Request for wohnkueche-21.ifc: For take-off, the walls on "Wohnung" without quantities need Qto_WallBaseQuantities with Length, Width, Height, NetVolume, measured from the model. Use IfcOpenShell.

First a look at what the model holds.

```python
import ifcopenshell
import ifcopenshell.util.element
import ifcopenshell.util.unit

model = ifcopenshell.open("wohnkueche-21.ifc")
print(model.schema)
for unit_type in ("LENGTHUNIT", "AREAUNIT", "VOLUMEUNIT"):
    print(unit_type, ifcopenshell.util.unit.calculate_unit_scale(model, unit_type))
storey = next(s for s in model.by_type("IfcBuildingStorey") if s.Name == "Wohnung")
walls = [e for e in ifcopenshell.util.element.get_decomposition(storey) if e.is_a("IfcWall")]
for e in sorted(walls, key=lambda e: e.id()):
    print(e.id(), e.is_a(), e.Name, list(ifcopenshell.util.element.get_psets(e, qtos_only=True)), sep=" | ")
```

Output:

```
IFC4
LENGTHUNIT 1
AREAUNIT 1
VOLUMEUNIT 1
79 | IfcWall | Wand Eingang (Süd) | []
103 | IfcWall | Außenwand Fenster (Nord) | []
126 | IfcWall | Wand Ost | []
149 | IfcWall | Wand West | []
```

```python
import ifcopenshell
import ifcopenshell.api.pset
import ifcopenshell.geom
import ifcopenshell.util.element
import ifcopenshell.util.shape
import ifcopenshell.util.unit

model = ifcopenshell.open("wohnkueche-21.ifc")
unit_scale = ifcopenshell.util.unit.calculate_unit_scale(model)
volume_scale = ifcopenshell.util.unit.calculate_unit_scale(model, "VOLUMEUNIT")
settings = ifcopenshell.geom.settings()

storey = next(s for s in model.by_type("IfcBuildingStorey") if s.Name == "Wohnung")
walls = [e for e in ifcopenshell.util.element.get_decomposition(storey) if e.is_a("IfcWall")]

for e in sorted(walls, key=lambda e: e.id()):
    if ifcopenshell.util.element.get_psets(e, qtos_only=True, should_inherit=False):
        continue
    # Geometry comes back in metres, in the element's own axes.
    shape = ifcopenshell.geom.create_shape(settings, e)
    values = {
        "Length": ifcopenshell.util.shape.get_x(shape.geometry) / unit_scale,
        "Width": ifcopenshell.util.shape.get_y(shape.geometry) / unit_scale,
        "Height": ifcopenshell.util.shape.get_z(shape.geometry) / unit_scale,
        "NetVolume": ifcopenshell.util.shape.get_volume(shape.geometry) / volume_scale,
    }
    qto = ifcopenshell.api.pset.add_qto(model, product=e, name="Qto_WallBaseQuantities")
    ifcopenshell.api.pset.edit_qto(model, qto=qto, properties=values)
    print(e.id(), {k: round(v, 3) for k, v in values.items()})

model.write("wohnkueche-21_v2.ifc")
```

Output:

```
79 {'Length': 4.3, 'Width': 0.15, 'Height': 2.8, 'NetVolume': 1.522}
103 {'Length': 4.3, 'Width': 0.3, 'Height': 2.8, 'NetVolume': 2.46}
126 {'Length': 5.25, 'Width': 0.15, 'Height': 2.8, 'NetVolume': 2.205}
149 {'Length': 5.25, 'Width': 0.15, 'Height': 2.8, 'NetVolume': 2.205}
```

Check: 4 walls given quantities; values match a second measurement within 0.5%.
